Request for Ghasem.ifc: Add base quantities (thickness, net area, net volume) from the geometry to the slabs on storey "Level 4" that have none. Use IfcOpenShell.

First a look at what the model holds.

```python
import ifcopenshell
import ifcopenshell.util.element
import ifcopenshell.util.unit

model = ifcopenshell.open("Ghasem.ifc")
print(model.schema)
for unit_type in ("LENGTHUNIT", "AREAUNIT", "VOLUMEUNIT"):
    print(unit_type, ifcopenshell.util.unit.calculate_unit_scale(model, unit_type))
storey = next(s for s in model.by_type("IfcBuildingStorey") if s.Name == "Level 4")
slabs = [e for e in ifcopenshell.util.element.get_decomposition(storey) if e.is_a("IfcSlab")]
for e in sorted(slabs, key=lambda e: e.id()):
    print(e.id(), e.is_a(), e.Name, list(ifcopenshell.util.element.get_psets(e, qtos_only=True)), sep=" | ")
```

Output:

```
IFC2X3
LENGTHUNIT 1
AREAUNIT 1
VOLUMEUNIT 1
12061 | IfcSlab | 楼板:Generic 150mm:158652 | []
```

```python
import ifcopenshell
import ifcopenshell.api.pset
import ifcopenshell.geom
import ifcopenshell.util.element
import ifcopenshell.util.shape
import ifcopenshell.util.unit

model = ifcopenshell.open("Ghasem.ifc")
unit_scale = ifcopenshell.util.unit.calculate_unit_scale(model)
area_scale = ifcopenshell.util.unit.calculate_unit_scale(model, "AREAUNIT")
volume_scale = ifcopenshell.util.unit.calculate_unit_scale(model, "VOLUMEUNIT")
settings = ifcopenshell.geom.settings()

storey = next(s for s in model.by_type("IfcBuildingStorey") if s.Name == "Level 4")
slabs = [e for e in ifcopenshell.util.element.get_decomposition(storey) if e.is_a("IfcSlab")]

for e in sorted(slabs, key=lambda e: e.id()):
    if ifcopenshell.util.element.get_psets(e, qtos_only=True, should_inherit=False):
        continue
    # Geometry comes back in metres, in the element's own axes.
    shape = ifcopenshell.geom.create_shape(settings, e)
    values = {
        "Width": ifcopenshell.util.shape.get_z(shape.geometry) / unit_scale,
        "NetArea": ifcopenshell.util.shape.get_footprint_area(shape.geometry) / area_scale,
        "NetVolume": ifcopenshell.util.shape.get_volume(shape.geometry) / volume_scale,
    }
    qto = ifcopenshell.api.pset.add_qto(model, product=e, name="BaseQuantities")
    ifcopenshell.api.pset.edit_qto(model, qto=qto, properties=values)
    print(e.id(), {k: round(v, 3) for k, v in values.items()})

model.write("Ghasem_updated.ifc")
```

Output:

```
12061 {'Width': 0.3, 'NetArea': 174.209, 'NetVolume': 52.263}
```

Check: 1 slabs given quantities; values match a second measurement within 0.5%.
